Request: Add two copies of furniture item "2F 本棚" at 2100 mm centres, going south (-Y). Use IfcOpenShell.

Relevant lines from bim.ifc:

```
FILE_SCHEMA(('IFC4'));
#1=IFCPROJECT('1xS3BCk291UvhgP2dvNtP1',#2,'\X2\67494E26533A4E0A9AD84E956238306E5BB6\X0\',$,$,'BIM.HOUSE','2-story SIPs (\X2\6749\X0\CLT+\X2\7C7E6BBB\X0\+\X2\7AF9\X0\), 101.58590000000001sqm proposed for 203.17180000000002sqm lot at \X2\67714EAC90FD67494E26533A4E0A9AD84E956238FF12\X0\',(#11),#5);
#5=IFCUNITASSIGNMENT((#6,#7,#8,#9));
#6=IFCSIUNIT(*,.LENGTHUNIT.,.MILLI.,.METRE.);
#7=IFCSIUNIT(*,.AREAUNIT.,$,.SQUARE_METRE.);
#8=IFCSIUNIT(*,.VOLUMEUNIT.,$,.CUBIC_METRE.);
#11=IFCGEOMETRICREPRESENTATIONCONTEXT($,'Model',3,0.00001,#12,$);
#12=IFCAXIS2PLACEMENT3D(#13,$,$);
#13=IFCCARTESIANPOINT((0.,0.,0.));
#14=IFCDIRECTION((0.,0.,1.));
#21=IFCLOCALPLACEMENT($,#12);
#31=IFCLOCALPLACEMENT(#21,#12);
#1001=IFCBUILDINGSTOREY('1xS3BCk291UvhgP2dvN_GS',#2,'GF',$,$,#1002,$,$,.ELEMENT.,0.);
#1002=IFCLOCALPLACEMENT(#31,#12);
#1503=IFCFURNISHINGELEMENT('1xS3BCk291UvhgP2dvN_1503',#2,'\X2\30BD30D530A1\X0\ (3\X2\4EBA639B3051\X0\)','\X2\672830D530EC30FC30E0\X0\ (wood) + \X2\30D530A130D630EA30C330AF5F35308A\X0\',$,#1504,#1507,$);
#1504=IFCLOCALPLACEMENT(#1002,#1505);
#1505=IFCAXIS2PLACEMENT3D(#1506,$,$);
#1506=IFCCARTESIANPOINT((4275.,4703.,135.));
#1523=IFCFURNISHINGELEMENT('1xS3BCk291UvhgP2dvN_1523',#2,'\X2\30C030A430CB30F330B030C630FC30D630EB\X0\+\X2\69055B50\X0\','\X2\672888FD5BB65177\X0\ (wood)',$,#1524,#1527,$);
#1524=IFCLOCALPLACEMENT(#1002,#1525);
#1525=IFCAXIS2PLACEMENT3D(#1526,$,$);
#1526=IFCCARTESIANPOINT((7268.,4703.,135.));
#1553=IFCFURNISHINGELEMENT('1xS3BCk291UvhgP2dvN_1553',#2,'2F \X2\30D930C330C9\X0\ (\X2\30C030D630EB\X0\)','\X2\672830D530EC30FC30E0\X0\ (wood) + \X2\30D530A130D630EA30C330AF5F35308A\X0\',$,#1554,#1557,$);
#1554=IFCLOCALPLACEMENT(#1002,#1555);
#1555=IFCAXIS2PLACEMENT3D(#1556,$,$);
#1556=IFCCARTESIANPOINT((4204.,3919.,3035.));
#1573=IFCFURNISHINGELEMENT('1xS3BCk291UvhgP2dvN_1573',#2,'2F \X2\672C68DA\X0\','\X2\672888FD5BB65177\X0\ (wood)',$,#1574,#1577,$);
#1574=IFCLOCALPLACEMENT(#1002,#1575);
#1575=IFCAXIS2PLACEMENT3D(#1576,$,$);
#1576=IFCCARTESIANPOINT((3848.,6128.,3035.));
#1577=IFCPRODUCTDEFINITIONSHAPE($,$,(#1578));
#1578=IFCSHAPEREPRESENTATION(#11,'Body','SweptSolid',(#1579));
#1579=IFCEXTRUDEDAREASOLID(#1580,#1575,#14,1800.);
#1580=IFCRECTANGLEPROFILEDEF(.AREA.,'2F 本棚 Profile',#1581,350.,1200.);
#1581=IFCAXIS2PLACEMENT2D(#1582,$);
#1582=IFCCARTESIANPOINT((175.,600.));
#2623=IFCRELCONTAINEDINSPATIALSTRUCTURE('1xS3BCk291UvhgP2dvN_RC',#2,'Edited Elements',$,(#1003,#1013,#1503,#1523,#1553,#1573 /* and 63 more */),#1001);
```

```python
import numpy as np
import ifcopenshell
import ifcopenshell.api.geometry
import ifcopenshell.api.root
import ifcopenshell.util.element
import ifcopenshell.util.placement
import ifcopenshell.util.unit

model = ifcopenshell.open("bim.ifc")
unit_scale = ifcopenshell.util.unit.calculate_unit_scale(model)


def reuse_history(source, copy):
    """copy_class also copies each property set's owner history, people and application; keep the originals."""
    for rel in copy.IsDefinedBy:
        if rel.is_a("IfcRelDefinesByProperties") and (history := rel.RelatingPropertyDefinition.OwnerHistory):
            rel.RelatingPropertyDefinition.OwnerHistory = source.OwnerHistory
            ifcopenshell.util.element.remove_deep2(model, history)


source = model.by_guid("1xS3BCk291UvhgP2dvN_1573")
base = ifcopenshell.util.placement.get_local_placement(source.ObjectPlacement)
step = np.array([0.0, -1.0, 0.0]) * 2.1 / unit_scale

for i in range(1, 3):
    copy = ifcopenshell.api.root.copy_class(model, product=source)
    copy.Representation = ifcopenshell.util.element.copy_deep(
        model, source.Representation, exclude=["IfcGeometricRepresentationContext", "IfcRepresentationMap"]
    )
    reuse_history(source, copy)
    matrix = base.copy()
    matrix[:3, 3] += i * step
    print("added at", matrix[:3, 3].round(3) + 0.0)
    ifcopenshell.api.geometry.edit_object_placement(model, product=copy, matrix=matrix, is_si=False)

model.write("bim-out.ifc")
```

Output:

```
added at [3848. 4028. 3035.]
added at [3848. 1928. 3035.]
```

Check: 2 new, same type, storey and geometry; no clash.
